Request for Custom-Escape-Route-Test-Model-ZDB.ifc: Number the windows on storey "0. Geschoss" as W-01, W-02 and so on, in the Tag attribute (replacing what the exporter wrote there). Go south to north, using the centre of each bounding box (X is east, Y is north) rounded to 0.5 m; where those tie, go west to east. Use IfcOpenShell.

First a look at what the model holds.

```python
import ifcopenshell
import ifcopenshell.util.element
import ifcopenshell.util.placement

model = ifcopenshell.open("Custom-Escape-Route-Test-Model-ZDB.ifc")
print(model.schema)
storey = next(s for s in model.by_type("IfcBuildingStorey") if s.Name == "0. Geschoss")
windows = [e for e in ifcopenshell.util.element.get_decomposition(storey) if e.is_a("IfcWindow")]
for e in sorted(windows, key=lambda e: e.id()):
    origin = ifcopenshell.util.placement.get_local_placement(e.ObjectPlacement)[:3, 3]
    print(e.id(), e.Tag, e.Name, origin.round(2) + 0.0, sep=" | ")
```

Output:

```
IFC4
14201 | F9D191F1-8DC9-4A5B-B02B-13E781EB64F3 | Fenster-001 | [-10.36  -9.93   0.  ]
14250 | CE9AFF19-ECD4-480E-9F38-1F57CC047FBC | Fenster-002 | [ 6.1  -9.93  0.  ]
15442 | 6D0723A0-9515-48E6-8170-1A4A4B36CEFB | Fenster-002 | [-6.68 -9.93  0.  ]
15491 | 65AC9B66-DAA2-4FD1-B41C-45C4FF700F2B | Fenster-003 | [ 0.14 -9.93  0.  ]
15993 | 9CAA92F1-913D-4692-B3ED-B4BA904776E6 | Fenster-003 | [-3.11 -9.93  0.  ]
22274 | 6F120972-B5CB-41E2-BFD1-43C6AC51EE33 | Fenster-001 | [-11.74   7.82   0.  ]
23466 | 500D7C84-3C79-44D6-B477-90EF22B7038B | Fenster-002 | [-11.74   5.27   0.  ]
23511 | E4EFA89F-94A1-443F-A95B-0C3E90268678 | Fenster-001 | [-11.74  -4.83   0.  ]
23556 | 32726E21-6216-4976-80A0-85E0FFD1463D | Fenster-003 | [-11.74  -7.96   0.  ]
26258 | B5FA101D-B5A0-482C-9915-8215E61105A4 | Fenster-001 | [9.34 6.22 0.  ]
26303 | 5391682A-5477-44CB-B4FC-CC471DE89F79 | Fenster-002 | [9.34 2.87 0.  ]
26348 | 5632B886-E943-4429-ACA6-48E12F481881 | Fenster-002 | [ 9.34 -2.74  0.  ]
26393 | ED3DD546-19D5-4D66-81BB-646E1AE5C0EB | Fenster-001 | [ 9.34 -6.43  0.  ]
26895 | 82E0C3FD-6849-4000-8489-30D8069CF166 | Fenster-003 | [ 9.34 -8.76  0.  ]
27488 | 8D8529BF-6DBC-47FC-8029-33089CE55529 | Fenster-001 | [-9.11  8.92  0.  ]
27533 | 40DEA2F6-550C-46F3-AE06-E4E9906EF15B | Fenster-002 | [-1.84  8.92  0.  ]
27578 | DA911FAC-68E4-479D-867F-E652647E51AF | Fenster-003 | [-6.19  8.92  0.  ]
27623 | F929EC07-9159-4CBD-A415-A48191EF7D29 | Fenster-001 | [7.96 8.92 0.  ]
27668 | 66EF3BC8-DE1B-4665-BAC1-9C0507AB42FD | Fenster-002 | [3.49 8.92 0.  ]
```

```python
import ifcopenshell
import ifcopenshell.geom
import ifcopenshell.util.element
import ifcopenshell.util.shape

model = ifcopenshell.open("Custom-Escape-Route-Test-Model-ZDB.ifc")
settings = ifcopenshell.geom.settings()
settings.set("use-world-coords", True)


def centre(element):
    shape = ifcopenshell.geom.create_shape(settings, element)
    return ifcopenshell.util.shape.get_bbox_centroid(shape.geometry)


storey = next(s for s in model.by_type("IfcBuildingStorey") if s.Name == "0. Geschoss")
windows = [e for e in ifcopenshell.util.element.get_decomposition(storey) if e.is_a("IfcWindow")]

# Insertion points can sit at a corner or the storey origin, so sort by the geometry (in metres).
centres = {e: centre(e) for e in windows}
windows.sort(key=lambda e: (round(centres[e][1] / 0.5), centres[e][0]))

for i, e in enumerate(windows, start=1):
    number = f"W-{i:02d}"
    e.Tag = number
    print(e.id(), number)

model.write("Custom-Escape-Route-Test-Model-ZDB_rev.ifc")
```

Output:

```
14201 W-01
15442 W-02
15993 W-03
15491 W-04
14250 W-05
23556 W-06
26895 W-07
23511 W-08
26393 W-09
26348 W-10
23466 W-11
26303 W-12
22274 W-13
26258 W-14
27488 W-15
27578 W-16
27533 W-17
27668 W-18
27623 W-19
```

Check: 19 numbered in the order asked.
